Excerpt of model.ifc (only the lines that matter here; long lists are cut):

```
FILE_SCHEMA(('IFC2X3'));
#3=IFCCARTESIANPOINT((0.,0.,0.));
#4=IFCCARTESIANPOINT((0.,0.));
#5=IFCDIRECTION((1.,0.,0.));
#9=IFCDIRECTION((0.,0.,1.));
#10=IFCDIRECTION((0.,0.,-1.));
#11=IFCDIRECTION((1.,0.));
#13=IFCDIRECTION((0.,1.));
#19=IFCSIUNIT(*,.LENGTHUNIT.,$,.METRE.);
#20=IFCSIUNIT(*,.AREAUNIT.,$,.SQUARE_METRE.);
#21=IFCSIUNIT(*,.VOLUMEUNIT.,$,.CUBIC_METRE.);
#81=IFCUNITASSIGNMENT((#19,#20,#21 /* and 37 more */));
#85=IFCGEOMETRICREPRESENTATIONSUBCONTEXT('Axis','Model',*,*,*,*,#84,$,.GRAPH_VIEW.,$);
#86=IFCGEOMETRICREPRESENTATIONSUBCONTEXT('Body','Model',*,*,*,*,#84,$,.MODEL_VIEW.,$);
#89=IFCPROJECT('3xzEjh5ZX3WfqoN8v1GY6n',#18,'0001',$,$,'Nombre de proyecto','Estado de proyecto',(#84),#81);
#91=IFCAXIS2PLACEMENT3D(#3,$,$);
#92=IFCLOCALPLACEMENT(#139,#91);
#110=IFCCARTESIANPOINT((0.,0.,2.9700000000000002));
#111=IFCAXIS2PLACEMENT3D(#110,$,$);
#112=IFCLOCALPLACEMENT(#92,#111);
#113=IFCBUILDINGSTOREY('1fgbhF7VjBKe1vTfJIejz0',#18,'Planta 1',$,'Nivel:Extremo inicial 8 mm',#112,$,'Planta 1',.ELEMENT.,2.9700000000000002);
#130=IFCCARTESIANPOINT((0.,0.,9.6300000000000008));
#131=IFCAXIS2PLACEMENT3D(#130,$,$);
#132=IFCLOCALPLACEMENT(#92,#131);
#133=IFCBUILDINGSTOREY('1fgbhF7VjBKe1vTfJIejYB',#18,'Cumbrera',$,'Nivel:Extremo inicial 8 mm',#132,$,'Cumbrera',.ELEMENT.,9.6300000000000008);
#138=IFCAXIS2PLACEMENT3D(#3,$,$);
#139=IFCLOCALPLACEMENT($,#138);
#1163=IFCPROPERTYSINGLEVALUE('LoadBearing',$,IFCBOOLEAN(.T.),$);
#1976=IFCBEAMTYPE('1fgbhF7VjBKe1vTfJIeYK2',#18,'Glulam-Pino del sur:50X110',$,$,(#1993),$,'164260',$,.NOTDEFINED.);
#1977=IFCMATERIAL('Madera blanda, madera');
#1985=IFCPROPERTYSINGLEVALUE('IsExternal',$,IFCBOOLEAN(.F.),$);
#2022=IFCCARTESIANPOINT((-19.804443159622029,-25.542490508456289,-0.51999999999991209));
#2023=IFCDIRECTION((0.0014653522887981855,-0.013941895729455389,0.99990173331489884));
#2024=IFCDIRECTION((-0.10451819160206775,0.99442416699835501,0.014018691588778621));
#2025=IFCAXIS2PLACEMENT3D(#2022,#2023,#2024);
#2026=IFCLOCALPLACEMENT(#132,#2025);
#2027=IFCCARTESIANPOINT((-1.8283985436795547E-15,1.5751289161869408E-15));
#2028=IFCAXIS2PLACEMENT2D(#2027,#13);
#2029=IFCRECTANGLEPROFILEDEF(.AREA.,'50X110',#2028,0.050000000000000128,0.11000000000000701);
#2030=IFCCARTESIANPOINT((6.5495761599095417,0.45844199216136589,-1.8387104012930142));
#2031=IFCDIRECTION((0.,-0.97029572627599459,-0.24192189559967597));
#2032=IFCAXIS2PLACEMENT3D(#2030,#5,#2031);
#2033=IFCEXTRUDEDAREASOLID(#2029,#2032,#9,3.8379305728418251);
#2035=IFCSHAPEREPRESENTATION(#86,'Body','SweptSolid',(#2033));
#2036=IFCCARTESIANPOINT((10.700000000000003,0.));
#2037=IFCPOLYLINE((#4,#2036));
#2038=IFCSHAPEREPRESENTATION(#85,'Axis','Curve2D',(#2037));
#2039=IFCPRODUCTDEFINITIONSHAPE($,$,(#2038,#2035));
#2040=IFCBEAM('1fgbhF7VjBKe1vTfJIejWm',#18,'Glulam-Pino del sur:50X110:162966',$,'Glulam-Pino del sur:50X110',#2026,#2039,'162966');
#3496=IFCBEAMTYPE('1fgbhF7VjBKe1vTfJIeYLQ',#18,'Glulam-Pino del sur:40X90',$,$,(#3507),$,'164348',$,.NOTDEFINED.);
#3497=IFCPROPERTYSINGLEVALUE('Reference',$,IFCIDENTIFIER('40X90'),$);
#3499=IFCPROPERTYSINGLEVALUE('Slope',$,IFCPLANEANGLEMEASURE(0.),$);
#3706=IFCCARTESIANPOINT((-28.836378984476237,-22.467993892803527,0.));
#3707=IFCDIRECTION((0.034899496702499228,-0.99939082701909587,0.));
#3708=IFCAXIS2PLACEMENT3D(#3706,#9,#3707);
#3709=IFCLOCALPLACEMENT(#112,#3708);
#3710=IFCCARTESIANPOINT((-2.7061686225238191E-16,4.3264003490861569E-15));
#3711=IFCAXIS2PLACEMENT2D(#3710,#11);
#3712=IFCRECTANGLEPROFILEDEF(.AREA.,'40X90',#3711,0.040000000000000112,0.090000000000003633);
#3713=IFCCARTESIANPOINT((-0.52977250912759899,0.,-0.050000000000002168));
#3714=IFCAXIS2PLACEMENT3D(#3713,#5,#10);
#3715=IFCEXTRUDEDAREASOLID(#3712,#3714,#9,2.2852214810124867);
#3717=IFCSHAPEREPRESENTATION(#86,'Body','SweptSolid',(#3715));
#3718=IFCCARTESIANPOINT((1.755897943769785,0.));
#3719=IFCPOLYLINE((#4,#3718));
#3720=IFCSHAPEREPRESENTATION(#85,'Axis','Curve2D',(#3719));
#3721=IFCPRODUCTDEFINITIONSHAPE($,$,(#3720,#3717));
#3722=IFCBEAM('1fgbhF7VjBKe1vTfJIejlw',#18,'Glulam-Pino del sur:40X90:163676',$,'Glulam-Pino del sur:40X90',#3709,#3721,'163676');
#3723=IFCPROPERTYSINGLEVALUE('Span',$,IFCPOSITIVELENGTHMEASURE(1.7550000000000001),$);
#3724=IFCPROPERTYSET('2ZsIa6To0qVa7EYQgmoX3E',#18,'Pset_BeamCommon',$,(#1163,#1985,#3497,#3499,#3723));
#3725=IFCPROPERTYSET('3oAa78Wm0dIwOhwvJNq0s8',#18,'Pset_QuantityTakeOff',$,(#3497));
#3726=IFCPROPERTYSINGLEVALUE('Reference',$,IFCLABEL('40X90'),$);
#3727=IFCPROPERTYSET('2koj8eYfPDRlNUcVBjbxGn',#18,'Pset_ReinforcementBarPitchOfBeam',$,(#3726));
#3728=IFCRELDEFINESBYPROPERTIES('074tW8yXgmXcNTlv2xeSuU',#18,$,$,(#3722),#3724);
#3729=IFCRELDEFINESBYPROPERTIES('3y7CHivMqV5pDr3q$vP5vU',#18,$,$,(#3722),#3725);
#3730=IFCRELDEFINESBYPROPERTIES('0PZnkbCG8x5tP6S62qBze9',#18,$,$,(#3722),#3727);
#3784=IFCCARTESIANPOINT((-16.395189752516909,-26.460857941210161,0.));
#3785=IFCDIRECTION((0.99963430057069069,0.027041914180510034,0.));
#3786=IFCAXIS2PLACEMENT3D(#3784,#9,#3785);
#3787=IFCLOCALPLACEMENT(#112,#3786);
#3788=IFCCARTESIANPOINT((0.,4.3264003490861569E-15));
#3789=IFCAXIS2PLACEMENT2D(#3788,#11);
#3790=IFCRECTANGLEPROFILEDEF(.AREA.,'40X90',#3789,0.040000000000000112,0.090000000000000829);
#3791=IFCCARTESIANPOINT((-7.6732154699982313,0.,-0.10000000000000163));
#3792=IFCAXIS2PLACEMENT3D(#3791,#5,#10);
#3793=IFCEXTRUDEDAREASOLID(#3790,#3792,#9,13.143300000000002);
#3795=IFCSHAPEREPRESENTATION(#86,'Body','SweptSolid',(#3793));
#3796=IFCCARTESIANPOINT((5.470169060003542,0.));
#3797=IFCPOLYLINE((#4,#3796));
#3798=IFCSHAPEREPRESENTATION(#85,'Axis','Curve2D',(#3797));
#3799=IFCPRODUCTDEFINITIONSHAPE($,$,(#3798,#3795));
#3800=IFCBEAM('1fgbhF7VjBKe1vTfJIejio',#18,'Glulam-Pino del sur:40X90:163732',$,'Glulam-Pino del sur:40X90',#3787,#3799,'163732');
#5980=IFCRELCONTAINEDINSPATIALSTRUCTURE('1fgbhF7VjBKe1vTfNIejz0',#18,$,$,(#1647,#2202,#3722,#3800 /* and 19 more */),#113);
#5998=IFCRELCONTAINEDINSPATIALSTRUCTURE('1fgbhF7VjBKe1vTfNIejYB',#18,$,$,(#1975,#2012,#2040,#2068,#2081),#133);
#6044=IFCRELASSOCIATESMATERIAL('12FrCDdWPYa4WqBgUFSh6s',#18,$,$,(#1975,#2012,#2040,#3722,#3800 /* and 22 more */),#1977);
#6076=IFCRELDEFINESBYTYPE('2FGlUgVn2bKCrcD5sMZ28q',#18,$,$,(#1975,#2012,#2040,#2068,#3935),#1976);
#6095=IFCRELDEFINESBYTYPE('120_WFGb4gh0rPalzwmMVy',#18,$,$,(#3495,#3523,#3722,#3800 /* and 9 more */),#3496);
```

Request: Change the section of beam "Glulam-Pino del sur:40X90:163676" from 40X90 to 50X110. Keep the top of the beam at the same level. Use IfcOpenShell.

```python
import ifcopenshell
import ifcopenshell.api.pset
import ifcopenshell.api.type
import ifcopenshell.util.element
import ifcopenshell.util.representation

model = ifcopenshell.open("model.ifc")

member = model.by_guid("1fgbhF7VjBKe1vTfJIejlw")
source = next(p for p in model.by_type("IfcRectangleProfileDef") if p.ProfileName == "50X110")

body = ifcopenshell.util.representation.get_representation(member, "Model", "Body")
solid = body.Items[0]
old_profile = solid.SweptArea

# Copy the section's sizes but keep this member's own profile position.
profile = ifcopenshell.util.element.copy(model, source)
# Profiles are centred, so shift by half the change in depth to hold the top.
shift = (old_profile.XDim - profile.XDim) / 2
x, y = old_profile.Position.Location.Coordinates
up = (-1.0, 0.0)  # upwards, in the solid's own plane
location = model.createIfcCartesianPoint((x + up[0] * shift, y + up[1] * shift))
profile.Position = model.createIfcAxis2Placement2D(location, old_profile.Position.RefDirection)
solid.SweptArea = profile
if not model.get_total_inverses(old_profile):
    ifcopenshell.util.element.remove_deep2(model, old_profile)

new_type = model.by_id(1976)
ifcopenshell.api.type.assign_type(
    model, related_objects=[member], relating_type=new_type, should_map_representations=False
)
member.Name = member.Name.replace("40X90", "50X110")
member.ObjectType = "Glulam-Pino del sur:50X110"
pset = model.by_id(ifcopenshell.util.element.get_pset(member, "Pset_BeamCommon", should_inherit=False)["id"])
ifcopenshell.api.pset.edit_pset(model, pset=pset, properties={"Reference": "50X110"})
pset = model.by_id(ifcopenshell.util.element.get_pset(member, "Pset_QuantityTakeOff", should_inherit=False)["id"])
ifcopenshell.api.pset.edit_pset(model, pset=pset, properties={"Reference": "50X110"})
pset = model.by_id(ifcopenshell.util.element.get_pset(member, "Pset_ReinforcementBarPitchOfBeam", should_inherit=False)["id"])
ifcopenshell.api.pset.edit_pset(model, pset=pset, properties={"Reference": "50X110"})

print(solid.SweptArea)

model.write("model_rev.ifc")
```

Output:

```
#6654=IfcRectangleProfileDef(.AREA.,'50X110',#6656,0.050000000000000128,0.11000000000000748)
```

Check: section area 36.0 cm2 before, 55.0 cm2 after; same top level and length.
